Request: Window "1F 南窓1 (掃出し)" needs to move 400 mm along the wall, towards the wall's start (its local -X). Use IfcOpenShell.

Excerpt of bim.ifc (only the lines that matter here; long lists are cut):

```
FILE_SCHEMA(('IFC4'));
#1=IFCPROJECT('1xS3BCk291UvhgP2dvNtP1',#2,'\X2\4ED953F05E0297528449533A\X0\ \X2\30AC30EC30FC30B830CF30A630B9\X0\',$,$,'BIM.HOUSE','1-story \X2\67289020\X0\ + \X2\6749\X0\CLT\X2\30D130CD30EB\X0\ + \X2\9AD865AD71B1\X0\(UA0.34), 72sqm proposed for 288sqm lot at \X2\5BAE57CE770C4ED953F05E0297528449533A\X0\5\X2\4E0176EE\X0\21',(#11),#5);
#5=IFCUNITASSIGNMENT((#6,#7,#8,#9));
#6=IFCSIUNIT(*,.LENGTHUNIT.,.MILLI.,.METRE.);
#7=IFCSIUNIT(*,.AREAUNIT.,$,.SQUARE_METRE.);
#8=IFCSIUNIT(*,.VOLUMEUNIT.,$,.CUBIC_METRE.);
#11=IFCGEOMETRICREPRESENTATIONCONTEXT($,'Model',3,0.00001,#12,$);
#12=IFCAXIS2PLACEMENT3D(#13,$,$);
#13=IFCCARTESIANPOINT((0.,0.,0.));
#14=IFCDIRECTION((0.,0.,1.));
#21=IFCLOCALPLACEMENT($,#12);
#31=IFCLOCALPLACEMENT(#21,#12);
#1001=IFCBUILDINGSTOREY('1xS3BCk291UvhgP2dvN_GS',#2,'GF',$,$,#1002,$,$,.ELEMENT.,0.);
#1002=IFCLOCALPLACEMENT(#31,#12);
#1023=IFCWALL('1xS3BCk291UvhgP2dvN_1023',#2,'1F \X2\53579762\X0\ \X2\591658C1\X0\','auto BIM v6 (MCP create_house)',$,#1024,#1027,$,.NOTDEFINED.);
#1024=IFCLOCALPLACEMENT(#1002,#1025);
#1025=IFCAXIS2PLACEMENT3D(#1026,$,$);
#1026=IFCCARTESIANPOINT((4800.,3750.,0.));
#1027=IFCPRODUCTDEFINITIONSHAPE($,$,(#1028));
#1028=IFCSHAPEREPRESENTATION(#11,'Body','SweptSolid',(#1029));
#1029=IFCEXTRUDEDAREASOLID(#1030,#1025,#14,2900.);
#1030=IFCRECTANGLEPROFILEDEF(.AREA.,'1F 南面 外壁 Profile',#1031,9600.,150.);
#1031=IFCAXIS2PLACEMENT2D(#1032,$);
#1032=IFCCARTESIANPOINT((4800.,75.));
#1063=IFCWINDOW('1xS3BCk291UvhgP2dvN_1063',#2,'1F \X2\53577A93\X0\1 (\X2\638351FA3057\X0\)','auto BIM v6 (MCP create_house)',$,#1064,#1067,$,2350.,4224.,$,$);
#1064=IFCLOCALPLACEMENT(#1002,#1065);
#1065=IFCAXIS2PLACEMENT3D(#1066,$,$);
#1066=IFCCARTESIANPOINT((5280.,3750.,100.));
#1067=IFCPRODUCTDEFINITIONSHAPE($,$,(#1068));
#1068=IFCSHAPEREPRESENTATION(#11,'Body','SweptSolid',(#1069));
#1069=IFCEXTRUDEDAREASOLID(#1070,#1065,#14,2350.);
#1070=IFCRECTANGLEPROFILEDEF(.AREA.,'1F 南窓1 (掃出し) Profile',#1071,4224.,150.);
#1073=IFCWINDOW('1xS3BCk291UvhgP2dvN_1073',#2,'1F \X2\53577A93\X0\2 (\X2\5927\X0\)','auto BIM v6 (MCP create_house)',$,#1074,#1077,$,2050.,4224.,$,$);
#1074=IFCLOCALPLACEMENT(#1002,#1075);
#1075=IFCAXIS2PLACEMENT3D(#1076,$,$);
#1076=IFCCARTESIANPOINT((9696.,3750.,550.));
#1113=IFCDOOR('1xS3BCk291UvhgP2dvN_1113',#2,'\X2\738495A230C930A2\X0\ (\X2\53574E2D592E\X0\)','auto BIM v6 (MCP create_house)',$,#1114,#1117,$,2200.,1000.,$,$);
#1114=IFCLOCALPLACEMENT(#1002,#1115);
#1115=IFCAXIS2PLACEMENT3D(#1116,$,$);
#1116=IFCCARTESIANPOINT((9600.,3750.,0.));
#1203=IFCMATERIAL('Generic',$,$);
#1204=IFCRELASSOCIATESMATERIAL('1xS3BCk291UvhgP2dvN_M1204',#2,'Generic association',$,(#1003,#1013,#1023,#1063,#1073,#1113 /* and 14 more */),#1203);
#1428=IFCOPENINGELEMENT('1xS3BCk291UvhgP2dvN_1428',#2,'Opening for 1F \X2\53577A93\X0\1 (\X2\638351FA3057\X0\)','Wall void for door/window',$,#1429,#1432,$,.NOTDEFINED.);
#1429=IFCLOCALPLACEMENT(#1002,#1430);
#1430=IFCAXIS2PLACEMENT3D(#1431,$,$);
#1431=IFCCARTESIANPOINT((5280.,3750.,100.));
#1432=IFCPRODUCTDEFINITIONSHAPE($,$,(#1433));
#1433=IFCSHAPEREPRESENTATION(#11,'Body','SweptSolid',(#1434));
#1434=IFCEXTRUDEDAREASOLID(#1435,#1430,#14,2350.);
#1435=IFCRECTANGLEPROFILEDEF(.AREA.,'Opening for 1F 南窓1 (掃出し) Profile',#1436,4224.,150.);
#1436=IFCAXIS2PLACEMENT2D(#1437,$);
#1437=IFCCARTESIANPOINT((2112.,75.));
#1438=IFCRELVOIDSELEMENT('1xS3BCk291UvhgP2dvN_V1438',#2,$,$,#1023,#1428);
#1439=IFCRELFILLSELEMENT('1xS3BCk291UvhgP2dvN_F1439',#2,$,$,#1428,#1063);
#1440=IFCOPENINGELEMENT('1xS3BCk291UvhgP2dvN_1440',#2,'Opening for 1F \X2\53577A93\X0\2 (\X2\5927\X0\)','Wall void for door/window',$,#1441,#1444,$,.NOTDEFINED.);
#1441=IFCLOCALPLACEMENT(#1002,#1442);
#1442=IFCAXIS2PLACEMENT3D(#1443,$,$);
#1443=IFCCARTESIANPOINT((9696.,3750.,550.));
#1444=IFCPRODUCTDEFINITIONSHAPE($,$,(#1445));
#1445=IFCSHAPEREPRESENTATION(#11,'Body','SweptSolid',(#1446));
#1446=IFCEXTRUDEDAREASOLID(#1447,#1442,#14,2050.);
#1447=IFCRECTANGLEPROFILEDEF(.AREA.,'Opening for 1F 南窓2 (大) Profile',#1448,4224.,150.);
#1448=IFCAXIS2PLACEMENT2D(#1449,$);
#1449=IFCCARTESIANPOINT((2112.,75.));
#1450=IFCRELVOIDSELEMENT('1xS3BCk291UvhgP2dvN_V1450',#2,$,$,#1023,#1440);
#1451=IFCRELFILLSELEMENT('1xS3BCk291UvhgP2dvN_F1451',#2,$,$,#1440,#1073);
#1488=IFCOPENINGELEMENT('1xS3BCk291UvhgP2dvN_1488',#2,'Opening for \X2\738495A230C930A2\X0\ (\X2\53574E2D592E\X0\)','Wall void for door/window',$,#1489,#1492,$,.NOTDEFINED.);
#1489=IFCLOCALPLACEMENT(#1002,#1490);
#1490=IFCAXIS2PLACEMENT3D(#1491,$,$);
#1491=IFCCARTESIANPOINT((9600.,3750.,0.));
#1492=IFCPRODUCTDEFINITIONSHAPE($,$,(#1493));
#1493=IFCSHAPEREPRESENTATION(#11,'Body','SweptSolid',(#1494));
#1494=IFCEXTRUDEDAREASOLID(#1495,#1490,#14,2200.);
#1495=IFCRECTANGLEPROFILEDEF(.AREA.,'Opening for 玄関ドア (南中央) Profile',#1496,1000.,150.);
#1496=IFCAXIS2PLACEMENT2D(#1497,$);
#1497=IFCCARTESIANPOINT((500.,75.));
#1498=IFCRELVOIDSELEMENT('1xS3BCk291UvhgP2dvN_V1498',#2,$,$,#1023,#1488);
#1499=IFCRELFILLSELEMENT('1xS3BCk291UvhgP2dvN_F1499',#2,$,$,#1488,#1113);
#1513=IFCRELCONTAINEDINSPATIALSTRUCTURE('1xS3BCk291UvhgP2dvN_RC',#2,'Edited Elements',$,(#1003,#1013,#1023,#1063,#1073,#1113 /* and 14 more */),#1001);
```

```python
import ifcopenshell
import ifcopenshell.api.geometry
import ifcopenshell.util.placement
import ifcopenshell.util.unit

model = ifcopenshell.open("bim.ifc")
unit_scale = ifcopenshell.util.unit.calculate_unit_scale(model)

window = model.by_guid("1xS3BCk291UvhgP2dvN_1063")
opening = window.FillsVoids[0].RelatingOpeningElement
wall = opening.VoidsElements[0].RelatingBuildingElement

wall_matrix = ifcopenshell.util.placement.get_local_placement(wall.ObjectPlacement)
shift = wall_matrix[:3, 0] * -0.4 / unit_scale
before = ifcopenshell.util.placement.get_local_placement(window.ObjectPlacement)[:3, 3].copy()

# The window is not placed relative to its opening, so move both.
for product in (opening, window):
    matrix = ifcopenshell.util.placement.get_local_placement(product.ObjectPlacement)
    matrix[:3, 3] += shift
    ifcopenshell.api.geometry.edit_object_placement(model, product=product, matrix=matrix, is_si=False)

after = ifcopenshell.util.placement.get_local_placement(window.ObjectPlacement)[:3, 3]
print("window moved by", (after - before).round(3) + 0.0)

model.write("bim_rev.ifc")
```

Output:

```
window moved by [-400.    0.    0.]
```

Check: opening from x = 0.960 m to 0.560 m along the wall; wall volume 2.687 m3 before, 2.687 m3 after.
